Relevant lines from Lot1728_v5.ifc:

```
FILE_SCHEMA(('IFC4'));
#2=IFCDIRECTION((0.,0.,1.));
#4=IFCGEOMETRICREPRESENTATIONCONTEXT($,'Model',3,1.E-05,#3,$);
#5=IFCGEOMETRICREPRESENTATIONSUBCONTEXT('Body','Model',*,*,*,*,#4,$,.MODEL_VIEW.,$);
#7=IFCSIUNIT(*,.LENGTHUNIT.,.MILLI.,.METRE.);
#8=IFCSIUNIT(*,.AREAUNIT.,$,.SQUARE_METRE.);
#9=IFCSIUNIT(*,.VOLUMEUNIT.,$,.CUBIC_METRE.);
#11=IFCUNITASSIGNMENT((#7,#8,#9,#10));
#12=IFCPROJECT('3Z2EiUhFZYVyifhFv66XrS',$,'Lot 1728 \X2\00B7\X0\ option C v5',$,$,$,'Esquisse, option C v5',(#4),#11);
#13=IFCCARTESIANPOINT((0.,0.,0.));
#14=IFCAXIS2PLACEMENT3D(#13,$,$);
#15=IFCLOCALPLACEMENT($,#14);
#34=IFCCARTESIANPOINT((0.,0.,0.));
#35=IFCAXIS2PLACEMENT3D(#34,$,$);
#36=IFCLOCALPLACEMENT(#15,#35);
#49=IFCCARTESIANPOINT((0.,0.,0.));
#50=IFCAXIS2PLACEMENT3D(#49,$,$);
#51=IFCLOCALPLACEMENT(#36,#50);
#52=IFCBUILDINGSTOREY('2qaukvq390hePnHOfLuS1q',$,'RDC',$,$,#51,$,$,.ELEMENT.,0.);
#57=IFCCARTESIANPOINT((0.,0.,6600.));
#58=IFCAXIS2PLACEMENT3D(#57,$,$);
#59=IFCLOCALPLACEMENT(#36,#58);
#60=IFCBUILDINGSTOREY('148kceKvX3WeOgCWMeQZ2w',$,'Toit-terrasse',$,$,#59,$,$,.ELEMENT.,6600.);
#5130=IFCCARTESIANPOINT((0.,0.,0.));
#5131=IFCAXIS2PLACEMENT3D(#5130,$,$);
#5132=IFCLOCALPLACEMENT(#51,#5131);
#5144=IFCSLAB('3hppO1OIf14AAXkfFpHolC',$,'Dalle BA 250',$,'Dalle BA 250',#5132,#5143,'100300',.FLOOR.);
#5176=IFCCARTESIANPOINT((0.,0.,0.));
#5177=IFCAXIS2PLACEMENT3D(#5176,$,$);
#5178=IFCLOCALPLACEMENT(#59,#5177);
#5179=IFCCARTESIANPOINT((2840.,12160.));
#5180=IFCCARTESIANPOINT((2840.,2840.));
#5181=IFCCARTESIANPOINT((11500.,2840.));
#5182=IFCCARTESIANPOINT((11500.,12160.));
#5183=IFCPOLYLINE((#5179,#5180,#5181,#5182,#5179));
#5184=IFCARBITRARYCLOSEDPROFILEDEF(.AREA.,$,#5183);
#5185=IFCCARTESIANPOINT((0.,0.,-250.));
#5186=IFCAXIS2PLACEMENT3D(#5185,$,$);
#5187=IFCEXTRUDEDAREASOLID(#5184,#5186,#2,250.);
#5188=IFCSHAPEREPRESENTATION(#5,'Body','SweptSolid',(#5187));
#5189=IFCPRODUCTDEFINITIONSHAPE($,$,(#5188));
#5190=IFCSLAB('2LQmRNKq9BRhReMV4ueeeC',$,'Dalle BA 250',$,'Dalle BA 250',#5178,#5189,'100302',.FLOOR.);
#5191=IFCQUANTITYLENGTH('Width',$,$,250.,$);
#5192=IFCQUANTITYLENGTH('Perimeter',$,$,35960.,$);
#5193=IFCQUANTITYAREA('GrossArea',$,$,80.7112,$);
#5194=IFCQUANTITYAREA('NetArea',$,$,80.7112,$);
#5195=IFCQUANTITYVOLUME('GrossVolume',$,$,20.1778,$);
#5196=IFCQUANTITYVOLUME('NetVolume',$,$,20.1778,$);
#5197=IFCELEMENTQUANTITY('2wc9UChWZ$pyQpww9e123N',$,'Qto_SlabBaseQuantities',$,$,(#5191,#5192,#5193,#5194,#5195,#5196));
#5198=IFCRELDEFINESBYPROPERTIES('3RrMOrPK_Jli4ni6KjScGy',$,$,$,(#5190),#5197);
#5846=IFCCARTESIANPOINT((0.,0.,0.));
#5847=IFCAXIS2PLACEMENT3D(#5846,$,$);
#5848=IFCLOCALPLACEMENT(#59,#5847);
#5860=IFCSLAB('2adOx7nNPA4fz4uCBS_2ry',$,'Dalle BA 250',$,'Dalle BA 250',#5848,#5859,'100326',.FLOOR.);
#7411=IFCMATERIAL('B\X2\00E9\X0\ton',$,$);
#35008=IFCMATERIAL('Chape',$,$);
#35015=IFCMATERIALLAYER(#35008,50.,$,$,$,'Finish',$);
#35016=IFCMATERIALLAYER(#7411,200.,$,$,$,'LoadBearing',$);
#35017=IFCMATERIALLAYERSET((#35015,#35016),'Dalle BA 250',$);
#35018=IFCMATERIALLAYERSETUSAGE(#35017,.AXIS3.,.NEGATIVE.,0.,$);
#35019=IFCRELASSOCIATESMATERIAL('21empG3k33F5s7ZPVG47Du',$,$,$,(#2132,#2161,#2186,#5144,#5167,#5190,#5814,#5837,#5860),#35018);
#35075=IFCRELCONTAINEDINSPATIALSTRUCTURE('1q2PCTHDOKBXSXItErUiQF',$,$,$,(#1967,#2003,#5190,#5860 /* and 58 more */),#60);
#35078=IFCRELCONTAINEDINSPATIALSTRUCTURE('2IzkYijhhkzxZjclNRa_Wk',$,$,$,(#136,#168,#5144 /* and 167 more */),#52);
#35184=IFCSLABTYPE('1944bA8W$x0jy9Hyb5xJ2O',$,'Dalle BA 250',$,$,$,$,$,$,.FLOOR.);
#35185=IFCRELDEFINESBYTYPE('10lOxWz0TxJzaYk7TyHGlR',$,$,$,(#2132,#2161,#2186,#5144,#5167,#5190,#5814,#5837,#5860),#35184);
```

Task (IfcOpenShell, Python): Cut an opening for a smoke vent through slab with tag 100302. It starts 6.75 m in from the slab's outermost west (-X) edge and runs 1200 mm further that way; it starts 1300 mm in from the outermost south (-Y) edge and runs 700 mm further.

```python
import numpy as np
import ifcopenshell
import ifcopenshell.api.feature
import ifcopenshell.api.geometry
import ifcopenshell.api.pset
import ifcopenshell.api.root
import ifcopenshell.geom
import ifcopenshell.util.element
import ifcopenshell.util.placement
import ifcopenshell.util.representation
import ifcopenshell.util.shape
import ifcopenshell.util.unit

model = ifcopenshell.open("Lot1728_v5.ifc")
unit_scale = ifcopenshell.util.unit.calculate_unit_scale(model)
area_scale = ifcopenshell.util.unit.calculate_unit_scale(model, "AREAUNIT")
volume_scale = ifcopenshell.util.unit.calculate_unit_scale(model, "VOLUMEUNIT")
settings = ifcopenshell.geom.settings()


def volume(element):
    """Net volume in cubic metres, openings subtracted."""
    shape = ifcopenshell.geom.create_shape(settings, element)
    return ifcopenshell.util.shape.get_volume(shape.geometry)


slab = model.by_id(5190)
before = volume(slab)

# Extent in the slab's own axes, in metres. The edges named are its -X and -Y sides.
slab_shape = ifcopenshell.geom.create_shape(settings, slab)
vertices = ifcopenshell.util.shape.get_vertices(slab_shape.geometry)
x_min, y_min, bottom = vertices.min(axis=0)
top = vertices[:, 2].max()

opening = ifcopenshell.api.root.create_entity(model, ifc_class="IfcOpeningElement", name="Smoke vent opening", predefined_type="OPENING")
context = ifcopenshell.util.representation.get_context(model, "Model", "Body", "MODEL_VIEW")
width, depth = 1.2, 0.7
outline = [(0.0, 0.0), (width, 0.0), (width, depth), (0.0, depth), (0.0, 0.0)]
# Overshoot both faces by 50 mm so the cut is clean.
shape = ifcopenshell.api.geometry.add_slab_representation(
    model, context=context, depth=top - bottom + 0.1, polyline=outline
)
ifcopenshell.api.geometry.assign_representation(model, product=opening, representation=shape)

matrix = ifcopenshell.util.placement.get_local_placement(slab.ObjectPlacement)
matrix[:, 3] = matrix @ np.append(np.array([x_min + 6.75, y_min + 1.3, bottom - 0.05]) / unit_scale, 1.0)
ifcopenshell.api.geometry.edit_object_placement(model, product=opening, matrix=matrix, is_si=False)
ifcopenshell.api.feature.add_feature(model, feature=opening, element=slab)

after = volume(slab)

# Update the slab's stored quantities.
qto = model.by_id(ifcopenshell.util.element.get_pset(slab, "Qto_SlabBaseQuantities", should_inherit=False)["id"])
ifcopenshell.api.pset.edit_qto(model, qto=qto, properties={
    "NetArea": after / (top - bottom) / area_scale,
    "NetVolume": after / volume_scale,
})

print(f"slab volume {before:.3f} -> {after:.3f} m3")

model.write("Lot1728_v5_updated.ifc")
```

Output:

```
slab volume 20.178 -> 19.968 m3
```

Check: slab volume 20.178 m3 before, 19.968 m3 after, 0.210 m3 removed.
